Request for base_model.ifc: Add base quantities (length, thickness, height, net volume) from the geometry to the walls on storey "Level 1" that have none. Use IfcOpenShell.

First a look at what the model holds.

```python
import ifcopenshell
import ifcopenshell.util.element
import ifcopenshell.util.unit

model = ifcopenshell.open("base_model.ifc")
print(model.schema)
for unit_type in ("LENGTHUNIT", "AREAUNIT", "VOLUMEUNIT"):
    print(unit_type, ifcopenshell.util.unit.calculate_unit_scale(model, unit_type))
storey = next(s for s in model.by_type("IfcBuildingStorey") if s.Name == "Level 1")
walls = [e for e in ifcopenshell.util.element.get_decomposition(storey) if e.is_a("IfcWall")]
for e in sorted(walls, key=lambda e: e.id()):
    print(e.id(), e.is_a(), e.Name, list(ifcopenshell.util.element.get_psets(e, qtos_only=True)), sep=" | ")
```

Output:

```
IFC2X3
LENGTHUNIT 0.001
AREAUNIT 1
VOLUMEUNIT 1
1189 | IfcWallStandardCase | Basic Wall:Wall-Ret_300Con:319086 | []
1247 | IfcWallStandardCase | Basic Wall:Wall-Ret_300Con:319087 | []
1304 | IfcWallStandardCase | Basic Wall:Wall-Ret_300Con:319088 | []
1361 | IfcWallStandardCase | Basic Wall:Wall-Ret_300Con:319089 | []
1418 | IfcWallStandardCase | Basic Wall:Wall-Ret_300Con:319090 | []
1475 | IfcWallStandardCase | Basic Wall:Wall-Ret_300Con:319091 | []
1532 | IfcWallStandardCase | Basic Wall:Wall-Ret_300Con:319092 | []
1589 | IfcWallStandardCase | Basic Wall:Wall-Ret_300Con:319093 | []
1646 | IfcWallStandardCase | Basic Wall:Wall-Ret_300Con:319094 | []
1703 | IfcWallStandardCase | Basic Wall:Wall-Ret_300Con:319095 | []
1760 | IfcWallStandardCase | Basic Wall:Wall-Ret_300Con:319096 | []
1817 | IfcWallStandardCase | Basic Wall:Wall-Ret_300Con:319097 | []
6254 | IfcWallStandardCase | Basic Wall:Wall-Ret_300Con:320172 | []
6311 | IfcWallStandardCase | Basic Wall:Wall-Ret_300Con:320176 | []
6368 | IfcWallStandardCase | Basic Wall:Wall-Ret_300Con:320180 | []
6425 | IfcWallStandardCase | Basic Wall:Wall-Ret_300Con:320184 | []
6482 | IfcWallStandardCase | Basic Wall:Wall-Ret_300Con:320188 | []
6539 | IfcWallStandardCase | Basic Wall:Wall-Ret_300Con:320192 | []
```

```python
import ifcopenshell
import ifcopenshell.api.pset
import ifcopenshell.geom
import ifcopenshell.util.element
import ifcopenshell.util.shape
import ifcopenshell.util.unit

model = ifcopenshell.open("base_model.ifc")
unit_scale = ifcopenshell.util.unit.calculate_unit_scale(model)
volume_scale = ifcopenshell.util.unit.calculate_unit_scale(model, "VOLUMEUNIT")
settings = ifcopenshell.geom.settings()

storey = next(s for s in model.by_type("IfcBuildingStorey") if s.Name == "Level 1")
walls = [e for e in ifcopenshell.util.element.get_decomposition(storey) if e.is_a("IfcWall")]

for e in sorted(walls, key=lambda e: e.id()):
    if ifcopenshell.util.element.get_psets(e, qtos_only=True, should_inherit=False):
        continue
    # Geometry comes back in metres, in the element's own axes.
    shape = ifcopenshell.geom.create_shape(settings, e)
    values = {
        "Length": ifcopenshell.util.shape.get_x(shape.geometry) / unit_scale,
        "Width": ifcopenshell.util.shape.get_y(shape.geometry) / unit_scale,
        "Height": ifcopenshell.util.shape.get_z(shape.geometry) / unit_scale,
        "NetVolume": ifcopenshell.util.shape.get_volume(shape.geometry) / volume_scale,
    }
    qto = ifcopenshell.api.pset.add_qto(model, product=e, name="BaseQuantities")
    ifcopenshell.api.pset.edit_qto(model, qto=qto, properties=values)
    print(e.id(), {k: round(v, 3) for k, v in values.items()})

model.write("base_model_updated.ifc")
```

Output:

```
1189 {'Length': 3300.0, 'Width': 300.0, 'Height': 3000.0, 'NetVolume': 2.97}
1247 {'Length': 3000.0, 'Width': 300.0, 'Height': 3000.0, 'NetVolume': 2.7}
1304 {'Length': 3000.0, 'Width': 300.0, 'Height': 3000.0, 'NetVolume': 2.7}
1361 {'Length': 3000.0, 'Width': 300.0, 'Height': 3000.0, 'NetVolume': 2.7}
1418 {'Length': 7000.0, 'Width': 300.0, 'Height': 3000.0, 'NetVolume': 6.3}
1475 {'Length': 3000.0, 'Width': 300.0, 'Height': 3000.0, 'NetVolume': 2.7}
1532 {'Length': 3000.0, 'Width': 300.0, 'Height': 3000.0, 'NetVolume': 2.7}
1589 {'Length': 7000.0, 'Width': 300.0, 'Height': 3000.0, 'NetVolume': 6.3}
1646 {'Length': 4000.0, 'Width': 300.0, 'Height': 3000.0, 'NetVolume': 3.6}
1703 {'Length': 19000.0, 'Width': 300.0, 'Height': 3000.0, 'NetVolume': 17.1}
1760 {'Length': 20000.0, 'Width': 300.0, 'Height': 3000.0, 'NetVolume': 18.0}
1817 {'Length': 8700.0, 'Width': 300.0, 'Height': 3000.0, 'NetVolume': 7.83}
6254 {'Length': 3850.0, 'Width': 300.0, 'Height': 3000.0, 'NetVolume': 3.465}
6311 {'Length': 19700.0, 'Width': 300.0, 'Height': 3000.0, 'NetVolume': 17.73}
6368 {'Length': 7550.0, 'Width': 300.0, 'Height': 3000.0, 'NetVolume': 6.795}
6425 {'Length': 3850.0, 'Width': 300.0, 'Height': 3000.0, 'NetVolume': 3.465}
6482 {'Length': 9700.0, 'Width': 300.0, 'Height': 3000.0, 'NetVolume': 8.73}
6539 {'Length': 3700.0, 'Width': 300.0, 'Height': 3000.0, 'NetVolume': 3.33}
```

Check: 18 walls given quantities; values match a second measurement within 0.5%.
